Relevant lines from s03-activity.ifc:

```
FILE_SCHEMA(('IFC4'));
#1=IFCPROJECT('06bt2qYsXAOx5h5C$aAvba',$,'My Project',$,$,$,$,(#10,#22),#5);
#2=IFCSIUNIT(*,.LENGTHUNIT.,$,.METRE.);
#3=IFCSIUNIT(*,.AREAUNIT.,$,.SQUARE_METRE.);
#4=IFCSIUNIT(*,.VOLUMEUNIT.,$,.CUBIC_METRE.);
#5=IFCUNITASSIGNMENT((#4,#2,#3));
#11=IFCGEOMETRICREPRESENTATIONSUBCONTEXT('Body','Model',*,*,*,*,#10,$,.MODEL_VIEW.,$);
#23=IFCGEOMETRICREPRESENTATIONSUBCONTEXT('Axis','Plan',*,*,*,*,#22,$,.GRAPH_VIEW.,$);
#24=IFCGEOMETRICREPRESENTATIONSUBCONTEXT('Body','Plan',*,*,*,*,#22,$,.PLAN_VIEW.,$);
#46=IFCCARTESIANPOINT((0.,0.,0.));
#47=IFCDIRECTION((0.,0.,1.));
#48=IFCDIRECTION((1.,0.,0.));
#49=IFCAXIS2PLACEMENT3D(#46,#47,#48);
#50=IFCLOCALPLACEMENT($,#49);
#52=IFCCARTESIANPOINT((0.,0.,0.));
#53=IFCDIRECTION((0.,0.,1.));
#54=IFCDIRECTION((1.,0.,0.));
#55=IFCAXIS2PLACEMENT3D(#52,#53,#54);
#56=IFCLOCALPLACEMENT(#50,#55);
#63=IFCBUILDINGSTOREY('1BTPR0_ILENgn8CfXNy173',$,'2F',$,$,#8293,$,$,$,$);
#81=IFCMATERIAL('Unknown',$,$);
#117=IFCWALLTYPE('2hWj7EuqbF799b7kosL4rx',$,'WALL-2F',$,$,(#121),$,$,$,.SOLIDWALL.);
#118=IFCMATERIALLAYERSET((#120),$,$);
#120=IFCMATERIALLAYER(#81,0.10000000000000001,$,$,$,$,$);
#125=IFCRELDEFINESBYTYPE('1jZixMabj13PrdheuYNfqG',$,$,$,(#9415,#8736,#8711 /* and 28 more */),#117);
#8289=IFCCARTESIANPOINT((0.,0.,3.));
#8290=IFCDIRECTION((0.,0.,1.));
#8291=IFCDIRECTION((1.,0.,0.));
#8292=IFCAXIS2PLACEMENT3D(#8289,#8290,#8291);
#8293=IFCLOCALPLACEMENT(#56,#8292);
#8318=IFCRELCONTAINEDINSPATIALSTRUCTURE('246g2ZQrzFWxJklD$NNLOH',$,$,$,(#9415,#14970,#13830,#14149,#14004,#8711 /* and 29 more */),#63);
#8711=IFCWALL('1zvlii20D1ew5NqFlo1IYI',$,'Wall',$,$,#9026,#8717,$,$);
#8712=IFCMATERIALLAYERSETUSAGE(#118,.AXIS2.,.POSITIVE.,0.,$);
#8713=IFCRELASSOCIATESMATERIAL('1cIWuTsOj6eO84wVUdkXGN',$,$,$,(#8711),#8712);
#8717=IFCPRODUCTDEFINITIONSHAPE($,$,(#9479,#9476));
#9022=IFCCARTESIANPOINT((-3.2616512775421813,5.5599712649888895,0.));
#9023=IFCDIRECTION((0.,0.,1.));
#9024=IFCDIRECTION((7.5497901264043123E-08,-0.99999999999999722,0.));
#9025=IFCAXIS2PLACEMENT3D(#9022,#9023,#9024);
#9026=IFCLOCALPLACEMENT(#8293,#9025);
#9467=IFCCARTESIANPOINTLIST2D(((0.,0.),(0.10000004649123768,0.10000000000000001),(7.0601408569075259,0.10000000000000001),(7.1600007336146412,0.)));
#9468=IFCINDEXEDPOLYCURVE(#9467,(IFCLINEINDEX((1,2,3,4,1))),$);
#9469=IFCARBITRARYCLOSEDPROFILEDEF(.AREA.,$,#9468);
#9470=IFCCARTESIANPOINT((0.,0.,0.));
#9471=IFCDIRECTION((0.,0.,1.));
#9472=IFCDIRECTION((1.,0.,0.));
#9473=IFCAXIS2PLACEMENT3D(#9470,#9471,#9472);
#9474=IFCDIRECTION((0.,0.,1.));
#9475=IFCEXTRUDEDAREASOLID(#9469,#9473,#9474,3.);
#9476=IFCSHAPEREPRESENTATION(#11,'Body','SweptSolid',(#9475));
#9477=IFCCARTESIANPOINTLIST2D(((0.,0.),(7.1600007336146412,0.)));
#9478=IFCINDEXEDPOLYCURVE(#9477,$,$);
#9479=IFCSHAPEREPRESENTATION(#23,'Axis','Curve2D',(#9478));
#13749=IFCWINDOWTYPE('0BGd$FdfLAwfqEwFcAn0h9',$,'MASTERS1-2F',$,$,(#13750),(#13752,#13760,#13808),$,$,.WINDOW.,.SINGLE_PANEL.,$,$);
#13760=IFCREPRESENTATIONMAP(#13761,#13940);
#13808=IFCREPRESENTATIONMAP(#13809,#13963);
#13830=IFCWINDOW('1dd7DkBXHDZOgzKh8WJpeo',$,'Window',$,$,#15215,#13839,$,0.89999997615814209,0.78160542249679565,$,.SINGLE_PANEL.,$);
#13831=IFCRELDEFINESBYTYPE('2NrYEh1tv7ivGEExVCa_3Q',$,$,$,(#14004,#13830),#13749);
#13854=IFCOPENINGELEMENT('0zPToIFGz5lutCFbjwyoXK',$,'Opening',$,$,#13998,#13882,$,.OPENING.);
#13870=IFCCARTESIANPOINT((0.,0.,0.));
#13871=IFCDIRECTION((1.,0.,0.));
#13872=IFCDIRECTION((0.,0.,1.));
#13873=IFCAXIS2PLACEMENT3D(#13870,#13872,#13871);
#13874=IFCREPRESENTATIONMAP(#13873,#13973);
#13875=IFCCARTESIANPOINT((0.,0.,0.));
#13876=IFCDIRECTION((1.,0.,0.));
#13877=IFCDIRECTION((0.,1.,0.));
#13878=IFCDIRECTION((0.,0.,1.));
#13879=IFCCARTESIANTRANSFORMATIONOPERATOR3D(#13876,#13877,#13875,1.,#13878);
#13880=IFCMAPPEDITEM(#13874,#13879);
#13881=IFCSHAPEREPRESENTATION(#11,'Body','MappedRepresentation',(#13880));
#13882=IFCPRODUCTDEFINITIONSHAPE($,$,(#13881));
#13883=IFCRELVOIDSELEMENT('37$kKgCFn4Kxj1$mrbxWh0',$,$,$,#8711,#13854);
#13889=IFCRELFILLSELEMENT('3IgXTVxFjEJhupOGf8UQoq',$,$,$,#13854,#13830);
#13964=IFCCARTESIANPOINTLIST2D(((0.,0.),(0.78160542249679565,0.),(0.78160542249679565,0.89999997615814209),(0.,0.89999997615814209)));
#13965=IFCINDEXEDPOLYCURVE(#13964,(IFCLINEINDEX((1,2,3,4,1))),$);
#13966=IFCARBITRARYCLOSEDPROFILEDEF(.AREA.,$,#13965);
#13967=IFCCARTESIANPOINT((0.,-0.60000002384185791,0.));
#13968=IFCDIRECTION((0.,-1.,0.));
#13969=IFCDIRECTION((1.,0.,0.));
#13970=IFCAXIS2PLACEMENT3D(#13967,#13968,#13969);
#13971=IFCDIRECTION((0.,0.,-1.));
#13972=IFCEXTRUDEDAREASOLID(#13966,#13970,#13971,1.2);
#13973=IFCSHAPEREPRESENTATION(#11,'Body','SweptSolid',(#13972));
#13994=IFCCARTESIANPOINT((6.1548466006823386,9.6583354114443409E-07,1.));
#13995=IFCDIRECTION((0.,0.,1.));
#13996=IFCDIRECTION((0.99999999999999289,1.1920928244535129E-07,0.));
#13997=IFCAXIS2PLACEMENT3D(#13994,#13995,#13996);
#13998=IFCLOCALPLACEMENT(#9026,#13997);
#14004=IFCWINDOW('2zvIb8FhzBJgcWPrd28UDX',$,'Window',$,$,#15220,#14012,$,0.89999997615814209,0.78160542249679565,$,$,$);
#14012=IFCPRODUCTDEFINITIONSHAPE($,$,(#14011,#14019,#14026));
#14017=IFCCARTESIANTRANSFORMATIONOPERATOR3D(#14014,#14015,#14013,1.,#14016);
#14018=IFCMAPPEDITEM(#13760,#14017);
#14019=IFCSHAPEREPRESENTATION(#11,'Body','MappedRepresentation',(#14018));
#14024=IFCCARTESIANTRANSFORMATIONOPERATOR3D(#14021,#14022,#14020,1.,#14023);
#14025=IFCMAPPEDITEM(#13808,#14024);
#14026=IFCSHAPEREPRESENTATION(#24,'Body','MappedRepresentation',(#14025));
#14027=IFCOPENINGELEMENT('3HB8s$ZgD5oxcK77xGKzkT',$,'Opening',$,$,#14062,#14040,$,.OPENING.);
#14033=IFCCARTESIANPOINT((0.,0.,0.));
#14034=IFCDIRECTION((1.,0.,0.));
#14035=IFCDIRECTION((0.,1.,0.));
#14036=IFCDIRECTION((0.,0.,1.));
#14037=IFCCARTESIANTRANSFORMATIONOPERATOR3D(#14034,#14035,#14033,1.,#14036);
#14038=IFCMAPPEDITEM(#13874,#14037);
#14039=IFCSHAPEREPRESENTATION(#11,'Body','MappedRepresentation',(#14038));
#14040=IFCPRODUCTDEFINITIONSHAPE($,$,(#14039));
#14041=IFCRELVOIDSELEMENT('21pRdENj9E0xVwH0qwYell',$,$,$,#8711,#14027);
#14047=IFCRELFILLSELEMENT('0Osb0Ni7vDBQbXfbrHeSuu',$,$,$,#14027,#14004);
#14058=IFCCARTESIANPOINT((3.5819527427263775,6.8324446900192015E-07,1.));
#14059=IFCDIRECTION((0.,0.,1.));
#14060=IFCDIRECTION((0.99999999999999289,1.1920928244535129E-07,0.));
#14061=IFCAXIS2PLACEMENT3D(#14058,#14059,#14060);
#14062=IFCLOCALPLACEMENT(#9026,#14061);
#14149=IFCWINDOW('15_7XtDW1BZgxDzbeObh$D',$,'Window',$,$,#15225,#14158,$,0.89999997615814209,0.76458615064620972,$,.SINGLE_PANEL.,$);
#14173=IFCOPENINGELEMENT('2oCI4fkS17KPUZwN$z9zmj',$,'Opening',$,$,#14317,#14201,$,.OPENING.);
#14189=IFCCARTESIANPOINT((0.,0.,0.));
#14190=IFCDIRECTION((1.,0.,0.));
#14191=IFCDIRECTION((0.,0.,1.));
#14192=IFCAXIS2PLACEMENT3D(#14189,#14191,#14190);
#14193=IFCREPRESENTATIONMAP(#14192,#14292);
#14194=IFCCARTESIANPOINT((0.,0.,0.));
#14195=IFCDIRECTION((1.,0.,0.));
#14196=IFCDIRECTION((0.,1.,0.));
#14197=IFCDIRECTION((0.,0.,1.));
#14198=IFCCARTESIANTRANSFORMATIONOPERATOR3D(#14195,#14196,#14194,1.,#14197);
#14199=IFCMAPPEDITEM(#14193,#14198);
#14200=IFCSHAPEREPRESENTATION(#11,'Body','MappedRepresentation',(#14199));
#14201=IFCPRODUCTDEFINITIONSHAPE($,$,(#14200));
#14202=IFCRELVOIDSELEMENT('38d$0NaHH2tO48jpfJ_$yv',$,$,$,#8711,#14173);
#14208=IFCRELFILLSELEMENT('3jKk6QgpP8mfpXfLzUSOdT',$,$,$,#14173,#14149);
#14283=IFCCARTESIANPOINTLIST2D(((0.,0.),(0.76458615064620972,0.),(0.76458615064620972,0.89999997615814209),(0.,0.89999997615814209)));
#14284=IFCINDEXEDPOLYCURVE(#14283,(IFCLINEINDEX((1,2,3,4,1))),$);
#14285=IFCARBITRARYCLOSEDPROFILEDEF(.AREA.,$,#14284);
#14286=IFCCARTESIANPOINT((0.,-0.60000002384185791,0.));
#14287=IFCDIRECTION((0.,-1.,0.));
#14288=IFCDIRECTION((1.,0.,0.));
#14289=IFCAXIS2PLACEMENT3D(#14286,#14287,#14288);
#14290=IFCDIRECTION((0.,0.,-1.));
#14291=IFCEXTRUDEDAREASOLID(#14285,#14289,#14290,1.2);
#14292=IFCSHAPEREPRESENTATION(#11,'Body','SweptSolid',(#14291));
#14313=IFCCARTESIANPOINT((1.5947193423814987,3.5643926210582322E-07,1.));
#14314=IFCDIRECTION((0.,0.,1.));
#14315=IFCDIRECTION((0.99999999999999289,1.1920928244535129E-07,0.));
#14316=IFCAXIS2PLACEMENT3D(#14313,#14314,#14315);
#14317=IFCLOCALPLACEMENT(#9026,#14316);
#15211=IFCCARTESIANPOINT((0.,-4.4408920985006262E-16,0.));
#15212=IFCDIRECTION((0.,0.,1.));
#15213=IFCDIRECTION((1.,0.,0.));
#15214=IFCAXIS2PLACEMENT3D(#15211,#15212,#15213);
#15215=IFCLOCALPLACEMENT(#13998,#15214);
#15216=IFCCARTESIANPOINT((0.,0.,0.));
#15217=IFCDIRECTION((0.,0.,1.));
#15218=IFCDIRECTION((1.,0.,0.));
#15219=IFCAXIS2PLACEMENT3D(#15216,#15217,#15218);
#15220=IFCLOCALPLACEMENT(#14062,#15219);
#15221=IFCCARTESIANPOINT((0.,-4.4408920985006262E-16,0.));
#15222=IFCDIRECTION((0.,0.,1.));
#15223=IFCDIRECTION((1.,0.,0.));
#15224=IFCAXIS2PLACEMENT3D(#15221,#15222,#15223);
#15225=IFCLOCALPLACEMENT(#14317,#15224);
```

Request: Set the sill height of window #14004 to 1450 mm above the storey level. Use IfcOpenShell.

```python
import numpy as np
import ifcopenshell
import ifcopenshell.api.geometry
import ifcopenshell.geom
import ifcopenshell.util.element
import ifcopenshell.util.placement
import ifcopenshell.util.shape
import ifcopenshell.util.unit

model = ifcopenshell.open("s03-activity.ifc")
unit_scale = ifcopenshell.util.unit.calculate_unit_scale(model)

window = model.by_id(14004)
opening = window.FillsVoids[0].RelatingOpeningElement
storey = ifcopenshell.util.element.get_container(window, ifc_class="IfcBuildingStorey")
level = ifcopenshell.util.placement.get_local_placement(storey.ObjectPlacement)[2, 3]

# The opening's origin need not be at the sill, so measure its lowest point.
shape = ifcopenshell.geom.create_shape(ifcopenshell.geom.settings(), opening)
bottom = ifcopenshell.util.shape.get_shape_bottom_elevation(shape, shape.geometry) / unit_scale
dz = level + 1.45 - bottom

shift = np.array([0.0, 0.0, dz])
# The window is placed relative to its opening, so it follows when the opening moves.
matrix = ifcopenshell.util.placement.get_local_placement(opening.ObjectPlacement)
matrix[:3, 3] += shift
ifcopenshell.api.geometry.edit_object_placement(
    model, product=opening, matrix=matrix, is_si=False, should_transform_children=True
)

print(f"moved by {dz * unit_scale:+.3f} m")

model.write("s03-activity_v2.ifc")
```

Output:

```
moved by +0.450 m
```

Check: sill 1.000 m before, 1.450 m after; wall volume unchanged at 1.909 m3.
